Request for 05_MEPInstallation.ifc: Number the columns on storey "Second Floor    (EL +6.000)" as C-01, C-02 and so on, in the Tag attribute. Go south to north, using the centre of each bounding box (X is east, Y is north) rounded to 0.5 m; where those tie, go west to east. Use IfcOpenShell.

First a look at what the model holds.

```python
import ifcopenshell
import ifcopenshell.util.element
import ifcopenshell.util.placement

model = ifcopenshell.open("05_MEPInstallation.ifc")
print(model.schema)
storey = next(s for s in model.by_type("IfcBuildingStorey") if s.Name == "Second Floor    (EL +6.000)")
columns = [e for e in ifcopenshell.util.element.get_decomposition(storey) if e.is_a("IfcColumn")]
for e in sorted(columns, key=lambda e: e.id()):
    origin = ifcopenshell.util.placement.get_local_placement(e.ObjectPlacement)[:3, 3]
    print(e.id(), e.Tag, e.Name, origin.round(2) + 0.0, sep=" | ")
```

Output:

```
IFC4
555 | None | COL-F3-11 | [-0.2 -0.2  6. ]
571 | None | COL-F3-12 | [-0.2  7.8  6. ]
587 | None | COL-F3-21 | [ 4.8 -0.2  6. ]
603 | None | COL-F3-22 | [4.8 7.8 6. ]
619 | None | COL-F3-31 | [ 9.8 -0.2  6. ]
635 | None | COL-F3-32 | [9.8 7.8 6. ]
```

```python
import ifcopenshell
import ifcopenshell.geom
import ifcopenshell.util.element
import ifcopenshell.util.shape

model = ifcopenshell.open("05_MEPInstallation.ifc")
settings = ifcopenshell.geom.settings()
settings.set("use-world-coords", True)


def centre(element):
    shape = ifcopenshell.geom.create_shape(settings, element)
    return ifcopenshell.util.shape.get_bbox_centroid(shape.geometry)


storey = next(s for s in model.by_type("IfcBuildingStorey") if s.Name == "Second Floor    (EL +6.000)")
columns = [e for e in ifcopenshell.util.element.get_decomposition(storey) if e.is_a("IfcColumn")]

# Insertion points can sit at a corner or the storey origin, so sort by the geometry (in metres).
centres = {e: centre(e) for e in columns}
columns.sort(key=lambda e: (round(centres[e][1] / 0.5), centres[e][0]))

for i, e in enumerate(columns, start=1):
    number = f"C-{i:02d}"
    e.Tag = number
    print(e.id(), number)

model.write("05_MEPInstallation_edited.ifc")
```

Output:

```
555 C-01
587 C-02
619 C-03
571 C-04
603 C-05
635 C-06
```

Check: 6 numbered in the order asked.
